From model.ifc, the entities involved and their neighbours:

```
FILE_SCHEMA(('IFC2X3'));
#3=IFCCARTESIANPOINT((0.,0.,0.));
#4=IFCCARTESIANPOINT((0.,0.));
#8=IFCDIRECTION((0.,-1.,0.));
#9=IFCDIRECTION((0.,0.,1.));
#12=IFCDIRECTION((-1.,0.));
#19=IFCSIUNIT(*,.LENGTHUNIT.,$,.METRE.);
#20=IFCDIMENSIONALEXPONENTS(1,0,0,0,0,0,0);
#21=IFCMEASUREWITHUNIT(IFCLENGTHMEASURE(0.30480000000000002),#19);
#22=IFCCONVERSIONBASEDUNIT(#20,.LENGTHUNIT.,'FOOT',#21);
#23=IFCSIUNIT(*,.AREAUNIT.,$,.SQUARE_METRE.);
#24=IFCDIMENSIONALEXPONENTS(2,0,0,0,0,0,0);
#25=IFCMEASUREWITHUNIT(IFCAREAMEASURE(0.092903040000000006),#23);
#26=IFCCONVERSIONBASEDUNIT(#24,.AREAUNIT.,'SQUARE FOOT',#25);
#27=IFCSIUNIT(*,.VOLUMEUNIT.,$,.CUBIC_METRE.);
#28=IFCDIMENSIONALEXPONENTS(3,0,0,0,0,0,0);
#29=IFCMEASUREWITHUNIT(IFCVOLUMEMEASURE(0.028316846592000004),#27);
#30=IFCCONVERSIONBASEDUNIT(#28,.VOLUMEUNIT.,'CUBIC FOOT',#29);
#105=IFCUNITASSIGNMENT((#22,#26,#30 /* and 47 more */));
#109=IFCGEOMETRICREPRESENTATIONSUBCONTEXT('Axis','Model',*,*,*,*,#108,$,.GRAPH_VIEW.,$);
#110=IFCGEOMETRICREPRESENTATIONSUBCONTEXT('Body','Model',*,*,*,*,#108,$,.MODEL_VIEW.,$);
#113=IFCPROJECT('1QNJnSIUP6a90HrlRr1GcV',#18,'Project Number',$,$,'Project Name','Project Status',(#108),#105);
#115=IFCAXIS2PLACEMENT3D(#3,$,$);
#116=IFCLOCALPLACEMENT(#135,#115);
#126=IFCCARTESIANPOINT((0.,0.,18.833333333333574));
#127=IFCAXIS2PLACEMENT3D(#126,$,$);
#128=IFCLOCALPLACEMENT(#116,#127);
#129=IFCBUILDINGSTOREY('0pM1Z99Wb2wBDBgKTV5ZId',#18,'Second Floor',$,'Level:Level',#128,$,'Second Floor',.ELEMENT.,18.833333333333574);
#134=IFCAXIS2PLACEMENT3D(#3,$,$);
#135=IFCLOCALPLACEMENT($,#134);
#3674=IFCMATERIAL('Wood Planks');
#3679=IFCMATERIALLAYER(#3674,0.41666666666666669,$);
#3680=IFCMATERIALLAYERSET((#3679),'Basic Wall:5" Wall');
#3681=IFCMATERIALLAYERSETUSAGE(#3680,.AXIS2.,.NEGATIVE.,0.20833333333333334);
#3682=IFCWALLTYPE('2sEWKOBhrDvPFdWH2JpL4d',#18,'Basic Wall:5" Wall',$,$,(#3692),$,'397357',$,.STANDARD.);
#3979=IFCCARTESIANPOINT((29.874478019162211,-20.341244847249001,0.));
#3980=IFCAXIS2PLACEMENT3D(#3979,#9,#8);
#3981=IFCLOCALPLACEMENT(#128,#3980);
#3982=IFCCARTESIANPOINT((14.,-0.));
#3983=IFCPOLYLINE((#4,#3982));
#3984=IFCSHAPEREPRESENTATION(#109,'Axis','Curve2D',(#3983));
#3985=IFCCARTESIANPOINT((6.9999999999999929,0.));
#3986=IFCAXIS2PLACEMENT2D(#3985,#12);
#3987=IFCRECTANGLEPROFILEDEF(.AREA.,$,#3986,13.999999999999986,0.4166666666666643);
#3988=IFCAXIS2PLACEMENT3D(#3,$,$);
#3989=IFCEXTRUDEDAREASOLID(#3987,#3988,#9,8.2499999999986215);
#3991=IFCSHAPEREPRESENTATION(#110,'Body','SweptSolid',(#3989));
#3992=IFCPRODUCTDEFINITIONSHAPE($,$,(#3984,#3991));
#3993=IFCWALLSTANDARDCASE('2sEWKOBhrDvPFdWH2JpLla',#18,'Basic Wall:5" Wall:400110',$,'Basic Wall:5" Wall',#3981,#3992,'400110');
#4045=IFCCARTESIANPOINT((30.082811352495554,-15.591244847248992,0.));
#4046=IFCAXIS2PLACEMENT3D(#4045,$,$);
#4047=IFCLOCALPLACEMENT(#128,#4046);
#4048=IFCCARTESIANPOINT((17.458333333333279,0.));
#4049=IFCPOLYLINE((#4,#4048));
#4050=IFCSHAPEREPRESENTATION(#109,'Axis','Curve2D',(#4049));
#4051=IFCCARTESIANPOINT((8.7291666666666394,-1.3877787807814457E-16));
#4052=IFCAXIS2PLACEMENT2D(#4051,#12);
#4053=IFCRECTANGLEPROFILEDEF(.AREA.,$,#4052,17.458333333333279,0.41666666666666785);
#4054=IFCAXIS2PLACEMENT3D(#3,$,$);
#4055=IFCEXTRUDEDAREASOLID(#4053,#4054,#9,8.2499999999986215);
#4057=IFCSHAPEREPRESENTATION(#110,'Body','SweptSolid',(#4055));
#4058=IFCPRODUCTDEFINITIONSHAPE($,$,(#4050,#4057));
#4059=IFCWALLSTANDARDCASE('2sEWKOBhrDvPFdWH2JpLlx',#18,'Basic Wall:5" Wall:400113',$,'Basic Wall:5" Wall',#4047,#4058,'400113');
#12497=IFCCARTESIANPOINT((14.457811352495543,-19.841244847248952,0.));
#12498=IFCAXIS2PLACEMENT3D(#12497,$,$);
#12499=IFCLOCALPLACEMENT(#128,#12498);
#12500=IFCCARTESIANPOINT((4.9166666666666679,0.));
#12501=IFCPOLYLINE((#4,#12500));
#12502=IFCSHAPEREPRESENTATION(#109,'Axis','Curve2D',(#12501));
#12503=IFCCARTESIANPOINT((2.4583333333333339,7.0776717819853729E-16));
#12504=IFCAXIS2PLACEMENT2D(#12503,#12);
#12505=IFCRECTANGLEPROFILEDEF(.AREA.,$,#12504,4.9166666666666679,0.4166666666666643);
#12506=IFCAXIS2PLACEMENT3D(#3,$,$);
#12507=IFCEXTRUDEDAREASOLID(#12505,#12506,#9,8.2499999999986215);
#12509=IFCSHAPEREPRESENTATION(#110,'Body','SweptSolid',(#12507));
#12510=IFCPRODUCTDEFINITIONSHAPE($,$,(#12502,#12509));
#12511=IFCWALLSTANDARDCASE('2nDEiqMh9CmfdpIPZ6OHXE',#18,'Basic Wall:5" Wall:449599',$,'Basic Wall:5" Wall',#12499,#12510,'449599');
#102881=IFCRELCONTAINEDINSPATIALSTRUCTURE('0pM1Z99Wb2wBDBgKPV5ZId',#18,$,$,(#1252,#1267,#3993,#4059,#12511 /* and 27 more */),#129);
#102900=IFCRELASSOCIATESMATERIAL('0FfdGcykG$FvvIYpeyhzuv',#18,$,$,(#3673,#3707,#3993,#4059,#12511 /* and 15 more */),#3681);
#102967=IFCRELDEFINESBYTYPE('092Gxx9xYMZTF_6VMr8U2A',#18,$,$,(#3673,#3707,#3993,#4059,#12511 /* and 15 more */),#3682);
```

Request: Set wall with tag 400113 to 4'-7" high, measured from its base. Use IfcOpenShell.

```python
import ifcopenshell
import ifcopenshell.geom
import ifcopenshell.util.representation
import ifcopenshell.util.shape
import ifcopenshell.util.unit

model = ifcopenshell.open("model.ifc")
unit_scale = ifcopenshell.util.unit.calculate_unit_scale(model)
settings = ifcopenshell.geom.settings()


def volume(element):
    """Net volume in cubic metres, openings subtracted."""
    shape = ifcopenshell.geom.create_shape(settings, element)
    return ifcopenshell.util.shape.get_volume(shape.geometry)


wall = model.by_guid("2sEWKOBhrDvPFdWH2JpLlx")
before = volume(wall)

body = ifcopenshell.util.representation.get_representation(wall, "Model", "Body")
solid = body.Items[0]
old_height = solid.Depth
solid.Depth = 55 * 0.0254 / unit_scale
after = volume(wall)

print(f"height {old_height:g} -> {solid.Depth:g}, volume {before:.3f} -> {after:.3f} m3")

model.write("model_rev.ifc")
```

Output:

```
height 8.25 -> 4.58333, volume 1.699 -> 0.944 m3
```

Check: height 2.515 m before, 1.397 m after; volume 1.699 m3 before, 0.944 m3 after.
